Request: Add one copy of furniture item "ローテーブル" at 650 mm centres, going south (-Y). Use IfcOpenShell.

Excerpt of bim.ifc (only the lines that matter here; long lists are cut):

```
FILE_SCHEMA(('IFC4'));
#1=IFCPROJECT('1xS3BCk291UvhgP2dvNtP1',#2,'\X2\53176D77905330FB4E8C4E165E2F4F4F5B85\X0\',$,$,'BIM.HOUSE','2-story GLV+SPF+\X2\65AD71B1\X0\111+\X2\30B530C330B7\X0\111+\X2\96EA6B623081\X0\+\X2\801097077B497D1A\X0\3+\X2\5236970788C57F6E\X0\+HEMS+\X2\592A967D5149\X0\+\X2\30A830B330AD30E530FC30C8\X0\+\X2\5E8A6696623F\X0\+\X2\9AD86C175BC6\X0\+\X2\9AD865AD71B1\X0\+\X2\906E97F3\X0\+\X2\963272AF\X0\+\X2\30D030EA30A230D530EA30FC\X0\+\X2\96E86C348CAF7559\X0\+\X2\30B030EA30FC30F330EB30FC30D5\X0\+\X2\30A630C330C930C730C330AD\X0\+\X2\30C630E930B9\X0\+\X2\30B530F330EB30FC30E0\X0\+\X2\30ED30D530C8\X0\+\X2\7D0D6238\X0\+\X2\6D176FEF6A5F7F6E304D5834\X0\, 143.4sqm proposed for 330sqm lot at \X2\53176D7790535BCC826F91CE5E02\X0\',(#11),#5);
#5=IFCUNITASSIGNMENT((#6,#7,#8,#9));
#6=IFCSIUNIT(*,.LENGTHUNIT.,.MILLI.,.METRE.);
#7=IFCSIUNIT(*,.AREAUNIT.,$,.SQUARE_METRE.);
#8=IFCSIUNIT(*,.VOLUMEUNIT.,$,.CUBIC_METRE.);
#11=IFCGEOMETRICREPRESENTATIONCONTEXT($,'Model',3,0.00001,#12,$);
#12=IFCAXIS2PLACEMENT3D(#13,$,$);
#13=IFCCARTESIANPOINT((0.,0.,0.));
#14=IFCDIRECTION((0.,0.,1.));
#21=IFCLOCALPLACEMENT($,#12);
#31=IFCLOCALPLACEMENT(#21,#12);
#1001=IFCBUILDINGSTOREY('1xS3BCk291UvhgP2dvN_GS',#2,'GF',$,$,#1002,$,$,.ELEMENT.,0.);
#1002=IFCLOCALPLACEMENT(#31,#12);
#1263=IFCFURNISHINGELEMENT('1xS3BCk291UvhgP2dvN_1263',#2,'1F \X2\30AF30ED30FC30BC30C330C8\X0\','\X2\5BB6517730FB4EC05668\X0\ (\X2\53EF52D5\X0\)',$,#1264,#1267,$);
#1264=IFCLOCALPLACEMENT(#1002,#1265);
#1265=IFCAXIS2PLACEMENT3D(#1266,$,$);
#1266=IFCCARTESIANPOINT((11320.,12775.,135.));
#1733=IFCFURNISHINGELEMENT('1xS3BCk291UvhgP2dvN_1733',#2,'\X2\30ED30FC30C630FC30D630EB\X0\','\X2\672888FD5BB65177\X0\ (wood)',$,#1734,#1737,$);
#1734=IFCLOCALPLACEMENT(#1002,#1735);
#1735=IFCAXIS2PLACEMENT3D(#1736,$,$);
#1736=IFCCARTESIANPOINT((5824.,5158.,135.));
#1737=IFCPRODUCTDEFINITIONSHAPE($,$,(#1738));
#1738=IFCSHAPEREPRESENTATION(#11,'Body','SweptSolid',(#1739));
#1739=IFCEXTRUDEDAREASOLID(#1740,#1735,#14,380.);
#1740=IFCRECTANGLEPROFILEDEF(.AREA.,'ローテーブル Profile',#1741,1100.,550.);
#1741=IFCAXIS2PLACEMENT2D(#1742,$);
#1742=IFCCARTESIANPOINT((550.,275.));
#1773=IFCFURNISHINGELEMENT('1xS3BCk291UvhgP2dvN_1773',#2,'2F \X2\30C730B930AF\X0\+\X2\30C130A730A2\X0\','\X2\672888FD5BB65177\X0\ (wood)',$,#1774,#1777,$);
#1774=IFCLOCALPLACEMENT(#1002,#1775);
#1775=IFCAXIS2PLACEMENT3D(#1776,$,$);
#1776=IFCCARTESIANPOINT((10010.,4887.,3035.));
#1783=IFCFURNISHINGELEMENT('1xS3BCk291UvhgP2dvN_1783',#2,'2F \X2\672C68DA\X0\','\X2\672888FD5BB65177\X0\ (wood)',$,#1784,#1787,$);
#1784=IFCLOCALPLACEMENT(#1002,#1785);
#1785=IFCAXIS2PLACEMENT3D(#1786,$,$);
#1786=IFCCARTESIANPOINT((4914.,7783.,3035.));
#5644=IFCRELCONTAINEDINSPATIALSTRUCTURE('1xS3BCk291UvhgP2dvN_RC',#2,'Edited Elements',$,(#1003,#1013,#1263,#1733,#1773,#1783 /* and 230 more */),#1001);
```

```python
import numpy as np
import ifcopenshell
import ifcopenshell.api.geometry
import ifcopenshell.api.root
import ifcopenshell.util.element
import ifcopenshell.util.placement
import ifcopenshell.util.unit

model = ifcopenshell.open("bim.ifc")
unit_scale = ifcopenshell.util.unit.calculate_unit_scale(model)


def reuse_history(source, copy):
    """copy_class also copies each property set's owner history, people and application; keep the originals."""
    for rel in copy.IsDefinedBy:
        if rel.is_a("IfcRelDefinesByProperties") and (history := rel.RelatingPropertyDefinition.OwnerHistory):
            rel.RelatingPropertyDefinition.OwnerHistory = source.OwnerHistory
            ifcopenshell.util.element.remove_deep2(model, history)


source = model.by_guid("1xS3BCk291UvhgP2dvN_1733")
base = ifcopenshell.util.placement.get_local_placement(source.ObjectPlacement)
step = np.array([0.0, -1.0, 0.0]) * 0.65 / unit_scale

for i in range(1, 2):
    copy = ifcopenshell.api.root.copy_class(model, product=source)
    copy.Representation = ifcopenshell.util.element.copy_deep(
        model, source.Representation, exclude=["IfcGeometricRepresentationContext", "IfcRepresentationMap"]
    )
    reuse_history(source, copy)
    matrix = base.copy()
    matrix[:3, 3] += i * step
    print("added at", matrix[:3, 3].round(3) + 0.0)
    ifcopenshell.api.geometry.edit_object_placement(model, product=copy, matrix=matrix, is_si=False)

model.write("bim_rev.ifc")
```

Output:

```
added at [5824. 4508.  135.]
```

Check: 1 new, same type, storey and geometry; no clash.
